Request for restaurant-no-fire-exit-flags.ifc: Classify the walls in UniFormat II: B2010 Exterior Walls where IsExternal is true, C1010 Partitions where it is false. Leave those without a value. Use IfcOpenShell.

First a look at what the model holds.

```python
import ifcopenshell
import ifcopenshell.util.element

model = ifcopenshell.open("restaurant-no-fire-exit-flags.ifc")
print(model.schema)
print("classifications:", [c.Name for c in model.by_type("IfcClassification")])
values = [ifcopenshell.util.element.get_pset(e, "Pset_WallCommon", "IsExternal") for e in model.by_type("IfcWall")]
for value in (True, False, None):
    print("IsExternal", value, values.count(value))
```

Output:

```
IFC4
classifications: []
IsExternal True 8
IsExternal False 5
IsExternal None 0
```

```python
import ifcopenshell
import ifcopenshell.api.classification
import ifcopenshell.util.element

model = ifcopenshell.open("restaurant-no-fire-exit-flags.ifc")

system = ifcopenshell.api.classification.add_classification(model, classification="UniFormat II")

walls = model.by_type("IfcWall")
external = {e: ifcopenshell.util.element.get_pset(e, "Pset_WallCommon", "IsExternal") for e in walls}
for flag, code, name in ((True, "B2010", "Exterior Walls"), (False, "C1010", "Partitions")):
    products = [e for e in walls if external[e] is flag]
    ifcopenshell.api.classification.add_reference(
        model, products=products, classification=system, identification=code, name=name
    )
    print(code, len(products))

model.write("restaurant-no-fire-exit-flags_edited.ifc")
```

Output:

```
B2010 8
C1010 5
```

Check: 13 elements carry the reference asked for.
